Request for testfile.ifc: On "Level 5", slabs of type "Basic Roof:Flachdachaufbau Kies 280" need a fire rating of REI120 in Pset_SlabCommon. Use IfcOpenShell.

First a look at what the model holds.

```python
import ifcopenshell
import ifcopenshell.util.element

model = ifcopenshell.open("testfile.ifc")
print(model.schema)
storey = next(s for s in model.by_type("IfcBuildingStorey") if s.Name == "Level 5")
slabs = [e for e in ifcopenshell.util.element.get_decomposition(storey) if e.is_a("IfcSlab")]
seen = {}
for e in slabs:
    element_type = ifcopenshell.util.element.get_type(e)
    key = (element_type.Name if element_type != e and element_type else None, ifcopenshell.util.element.get_pset(e, "Pset_SlabCommon", "FireRating"))
    seen[key] = seen.get(key, 0) + 1
for (name, value), count in sorted(seen.items(), key=str):
    print(count, "x", name, "|", value)
```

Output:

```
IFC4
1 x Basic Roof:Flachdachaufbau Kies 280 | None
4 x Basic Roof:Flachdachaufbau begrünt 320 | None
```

```python
import ifcopenshell
import ifcopenshell.api.pset
import ifcopenshell.util.element

model = ifcopenshell.open("testfile.ifc")

storey = next(s for s in model.by_type("IfcBuildingStorey") if s.Name == "Level 5")
slabs = [e for e in ifcopenshell.util.element.get_decomposition(storey) if e.is_a("IfcSlab")]

count = 0
for e in slabs:
    element_type = ifcopenshell.util.element.get_type(e)
    if element_type in (None, e) or element_type.Name != "Basic Roof:Flachdachaufbau Kies 280":
        continue
    # add_pset returns the element's existing set when there is one.
    pset = ifcopenshell.api.pset.add_pset(model, product=e, name="Pset_SlabCommon")
    ifcopenshell.api.pset.edit_pset(model, pset=pset, properties={"FireRating": "REI120"})
    count += 1

print(count, "slabs updated")

model.write("testfile-out.ifc")
```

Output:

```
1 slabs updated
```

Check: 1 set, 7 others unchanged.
